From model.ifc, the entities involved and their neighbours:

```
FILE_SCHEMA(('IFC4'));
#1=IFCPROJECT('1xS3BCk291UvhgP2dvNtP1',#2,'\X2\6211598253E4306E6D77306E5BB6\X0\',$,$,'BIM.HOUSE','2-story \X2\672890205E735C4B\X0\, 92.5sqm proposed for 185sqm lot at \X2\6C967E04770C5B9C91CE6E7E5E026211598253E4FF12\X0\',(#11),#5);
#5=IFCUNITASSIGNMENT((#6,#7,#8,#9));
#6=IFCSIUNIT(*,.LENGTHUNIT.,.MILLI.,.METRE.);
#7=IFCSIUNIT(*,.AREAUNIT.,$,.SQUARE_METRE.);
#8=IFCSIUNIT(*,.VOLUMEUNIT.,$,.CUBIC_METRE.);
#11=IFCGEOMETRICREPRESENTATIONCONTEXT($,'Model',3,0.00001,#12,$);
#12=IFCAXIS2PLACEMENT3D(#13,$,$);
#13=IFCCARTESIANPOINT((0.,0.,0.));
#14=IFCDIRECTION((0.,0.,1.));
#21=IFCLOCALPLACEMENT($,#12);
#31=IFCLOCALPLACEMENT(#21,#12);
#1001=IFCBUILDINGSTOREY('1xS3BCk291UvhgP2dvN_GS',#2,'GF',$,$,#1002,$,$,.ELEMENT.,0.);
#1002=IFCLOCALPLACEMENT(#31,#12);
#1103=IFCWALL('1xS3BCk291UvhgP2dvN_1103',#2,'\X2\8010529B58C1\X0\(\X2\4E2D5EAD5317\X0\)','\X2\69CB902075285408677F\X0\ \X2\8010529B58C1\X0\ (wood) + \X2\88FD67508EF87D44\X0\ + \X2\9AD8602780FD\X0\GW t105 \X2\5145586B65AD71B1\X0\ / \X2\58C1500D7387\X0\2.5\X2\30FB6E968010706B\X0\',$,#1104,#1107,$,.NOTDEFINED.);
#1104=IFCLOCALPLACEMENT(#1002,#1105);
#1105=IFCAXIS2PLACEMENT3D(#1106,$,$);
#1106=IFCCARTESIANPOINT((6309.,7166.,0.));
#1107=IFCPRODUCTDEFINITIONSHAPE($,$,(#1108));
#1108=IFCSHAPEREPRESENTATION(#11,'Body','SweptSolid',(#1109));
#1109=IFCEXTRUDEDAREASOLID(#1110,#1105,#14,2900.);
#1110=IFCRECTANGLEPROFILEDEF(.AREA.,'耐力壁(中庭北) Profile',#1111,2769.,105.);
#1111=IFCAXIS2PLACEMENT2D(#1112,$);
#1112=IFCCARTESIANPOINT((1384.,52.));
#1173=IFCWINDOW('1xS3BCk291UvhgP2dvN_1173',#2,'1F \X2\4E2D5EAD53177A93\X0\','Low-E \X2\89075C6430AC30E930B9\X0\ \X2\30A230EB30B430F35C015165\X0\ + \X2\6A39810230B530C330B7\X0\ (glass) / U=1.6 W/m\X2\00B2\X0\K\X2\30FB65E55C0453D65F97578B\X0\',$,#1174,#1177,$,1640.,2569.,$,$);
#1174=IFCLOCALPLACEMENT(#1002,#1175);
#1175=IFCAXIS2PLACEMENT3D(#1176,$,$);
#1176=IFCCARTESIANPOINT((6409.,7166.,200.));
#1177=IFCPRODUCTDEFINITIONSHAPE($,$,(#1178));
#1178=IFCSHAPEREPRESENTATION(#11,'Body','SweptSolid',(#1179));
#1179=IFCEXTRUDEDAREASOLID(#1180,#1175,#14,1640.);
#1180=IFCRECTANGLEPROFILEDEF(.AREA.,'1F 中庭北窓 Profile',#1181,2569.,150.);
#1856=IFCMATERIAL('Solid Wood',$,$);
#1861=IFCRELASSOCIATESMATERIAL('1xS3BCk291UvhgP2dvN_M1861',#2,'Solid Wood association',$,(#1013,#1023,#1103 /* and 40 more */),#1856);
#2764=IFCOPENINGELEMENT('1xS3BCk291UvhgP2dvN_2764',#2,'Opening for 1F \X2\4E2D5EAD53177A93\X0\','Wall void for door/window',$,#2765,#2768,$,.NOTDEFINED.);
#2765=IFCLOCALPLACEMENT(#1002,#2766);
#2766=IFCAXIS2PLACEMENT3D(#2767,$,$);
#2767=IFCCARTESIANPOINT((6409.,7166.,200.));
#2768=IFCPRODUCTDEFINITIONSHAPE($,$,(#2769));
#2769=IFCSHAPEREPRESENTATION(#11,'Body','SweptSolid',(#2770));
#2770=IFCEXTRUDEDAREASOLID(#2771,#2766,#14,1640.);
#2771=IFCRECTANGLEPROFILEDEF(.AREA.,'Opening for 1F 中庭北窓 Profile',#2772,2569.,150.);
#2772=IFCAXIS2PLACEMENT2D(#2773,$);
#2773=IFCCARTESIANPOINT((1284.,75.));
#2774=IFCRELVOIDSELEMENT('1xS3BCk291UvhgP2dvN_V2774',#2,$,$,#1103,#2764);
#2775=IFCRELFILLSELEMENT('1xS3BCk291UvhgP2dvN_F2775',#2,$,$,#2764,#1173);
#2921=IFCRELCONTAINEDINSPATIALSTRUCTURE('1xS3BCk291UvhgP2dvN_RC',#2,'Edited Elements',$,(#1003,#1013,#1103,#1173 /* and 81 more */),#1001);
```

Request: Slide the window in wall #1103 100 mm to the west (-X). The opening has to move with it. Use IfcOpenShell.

```python
import ifcopenshell
import ifcopenshell.api.geometry
import ifcopenshell.util.placement

model = ifcopenshell.open("model.ifc")

window = model.by_guid("1xS3BCk291UvhgP2dvN_1173")
opening = window.FillsVoids[0].RelatingOpeningElement
wall = opening.VoidsElements[0].RelatingBuildingElement

wall_matrix = ifcopenshell.util.placement.get_local_placement(wall.ObjectPlacement)
shift = wall_matrix[:3, 0] * -100.0
before = ifcopenshell.util.placement.get_local_placement(window.ObjectPlacement)[:3, 3].copy()

# The window is not placed relative to its opening, so move both.
for product in (opening, window):
    matrix = ifcopenshell.util.placement.get_local_placement(product.ObjectPlacement)
    matrix[:3, 3] += shift
    ifcopenshell.api.geometry.edit_object_placement(model, product=product, matrix=matrix, is_si=False)

after = ifcopenshell.util.placement.get_local_placement(window.ObjectPlacement)[:3, 3]
print("window moved by", (after - before).round(3) + 0.0)

model.write("model_v2.ifc")
```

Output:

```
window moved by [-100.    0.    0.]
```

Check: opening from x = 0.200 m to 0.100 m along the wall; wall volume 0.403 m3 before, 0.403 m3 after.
